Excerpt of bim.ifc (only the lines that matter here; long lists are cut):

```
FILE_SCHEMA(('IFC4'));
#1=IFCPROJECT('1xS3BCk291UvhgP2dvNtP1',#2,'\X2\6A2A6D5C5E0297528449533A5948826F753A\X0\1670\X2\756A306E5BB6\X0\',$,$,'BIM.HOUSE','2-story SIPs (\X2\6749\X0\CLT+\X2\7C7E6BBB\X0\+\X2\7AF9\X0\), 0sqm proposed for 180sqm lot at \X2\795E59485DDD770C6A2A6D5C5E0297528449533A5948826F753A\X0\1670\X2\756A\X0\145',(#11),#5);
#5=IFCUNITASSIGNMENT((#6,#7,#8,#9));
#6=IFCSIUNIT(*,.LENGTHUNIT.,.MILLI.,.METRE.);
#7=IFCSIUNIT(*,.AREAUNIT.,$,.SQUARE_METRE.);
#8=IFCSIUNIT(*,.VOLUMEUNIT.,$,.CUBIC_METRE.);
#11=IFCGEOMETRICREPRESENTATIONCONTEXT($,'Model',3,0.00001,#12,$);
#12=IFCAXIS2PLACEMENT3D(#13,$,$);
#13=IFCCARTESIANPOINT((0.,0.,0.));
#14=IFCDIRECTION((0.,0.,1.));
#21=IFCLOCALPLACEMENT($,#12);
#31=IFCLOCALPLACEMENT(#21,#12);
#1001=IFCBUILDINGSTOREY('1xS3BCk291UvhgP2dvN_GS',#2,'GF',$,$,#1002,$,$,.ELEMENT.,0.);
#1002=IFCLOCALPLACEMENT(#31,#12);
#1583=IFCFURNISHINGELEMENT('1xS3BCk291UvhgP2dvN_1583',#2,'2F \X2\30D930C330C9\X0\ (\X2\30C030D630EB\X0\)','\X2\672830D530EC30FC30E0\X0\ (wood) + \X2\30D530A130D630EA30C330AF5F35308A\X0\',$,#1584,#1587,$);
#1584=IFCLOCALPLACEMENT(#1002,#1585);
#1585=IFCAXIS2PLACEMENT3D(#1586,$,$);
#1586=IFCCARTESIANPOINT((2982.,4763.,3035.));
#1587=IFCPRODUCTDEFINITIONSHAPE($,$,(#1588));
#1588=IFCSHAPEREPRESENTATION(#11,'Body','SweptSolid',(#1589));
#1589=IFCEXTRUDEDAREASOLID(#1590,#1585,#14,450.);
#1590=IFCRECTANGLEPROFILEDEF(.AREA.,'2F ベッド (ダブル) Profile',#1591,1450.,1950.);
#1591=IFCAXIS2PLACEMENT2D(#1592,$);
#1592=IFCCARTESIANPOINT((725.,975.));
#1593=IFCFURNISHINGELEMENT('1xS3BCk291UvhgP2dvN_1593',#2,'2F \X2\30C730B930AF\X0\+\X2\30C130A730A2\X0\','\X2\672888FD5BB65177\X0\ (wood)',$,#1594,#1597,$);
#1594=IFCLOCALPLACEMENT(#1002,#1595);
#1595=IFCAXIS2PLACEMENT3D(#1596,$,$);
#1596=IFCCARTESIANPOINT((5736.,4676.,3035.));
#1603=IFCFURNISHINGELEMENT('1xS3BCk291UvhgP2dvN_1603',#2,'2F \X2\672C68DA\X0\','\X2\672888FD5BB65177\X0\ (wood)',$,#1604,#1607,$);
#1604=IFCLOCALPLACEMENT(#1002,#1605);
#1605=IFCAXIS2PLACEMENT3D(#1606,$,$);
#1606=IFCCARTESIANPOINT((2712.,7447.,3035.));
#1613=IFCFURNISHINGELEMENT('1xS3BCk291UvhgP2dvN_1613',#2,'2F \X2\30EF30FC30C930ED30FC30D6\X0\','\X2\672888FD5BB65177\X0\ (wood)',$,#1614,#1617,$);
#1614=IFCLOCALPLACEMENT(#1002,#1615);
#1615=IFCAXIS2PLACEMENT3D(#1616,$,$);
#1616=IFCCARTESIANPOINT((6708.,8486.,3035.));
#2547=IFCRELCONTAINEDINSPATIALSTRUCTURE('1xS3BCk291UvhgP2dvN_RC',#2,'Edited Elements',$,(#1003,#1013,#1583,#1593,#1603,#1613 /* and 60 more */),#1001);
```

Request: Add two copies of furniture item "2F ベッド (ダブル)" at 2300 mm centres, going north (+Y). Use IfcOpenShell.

```python
import numpy as np
import ifcopenshell
import ifcopenshell.api.geometry
import ifcopenshell.api.root
import ifcopenshell.util.element
import ifcopenshell.util.placement
import ifcopenshell.util.unit

model = ifcopenshell.open("bim.ifc")
unit_scale = ifcopenshell.util.unit.calculate_unit_scale(model)


def reuse_history(source, copy):
    """copy_class also copies each property set's owner history, people and application; keep the originals."""
    for rel in copy.IsDefinedBy:
        if rel.is_a("IfcRelDefinesByProperties") and (history := rel.RelatingPropertyDefinition.OwnerHistory):
            rel.RelatingPropertyDefinition.OwnerHistory = source.OwnerHistory
            ifcopenshell.util.element.remove_deep2(model, history)


source = model.by_guid("1xS3BCk291UvhgP2dvN_1583")
base = ifcopenshell.util.placement.get_local_placement(source.ObjectPlacement)
step = np.array([0.0, 1.0, 0.0]) * 2.3 / unit_scale

for i in range(1, 3):
    copy = ifcopenshell.api.root.copy_class(model, product=source)
    copy.Representation = ifcopenshell.util.element.copy_deep(
        model, source.Representation, exclude=["IfcGeometricRepresentationContext", "IfcRepresentationMap"]
    )
    reuse_history(source, copy)
    matrix = base.copy()
    matrix[:3, 3] += i * step
    print("added at", matrix[:3, 3].round(3) + 0.0)
    ifcopenshell.api.geometry.edit_object_placement(model, product=copy, matrix=matrix, is_si=False)

model.write("bim_v2.ifc")
```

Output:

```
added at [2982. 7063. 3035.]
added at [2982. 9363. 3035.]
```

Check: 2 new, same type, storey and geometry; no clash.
